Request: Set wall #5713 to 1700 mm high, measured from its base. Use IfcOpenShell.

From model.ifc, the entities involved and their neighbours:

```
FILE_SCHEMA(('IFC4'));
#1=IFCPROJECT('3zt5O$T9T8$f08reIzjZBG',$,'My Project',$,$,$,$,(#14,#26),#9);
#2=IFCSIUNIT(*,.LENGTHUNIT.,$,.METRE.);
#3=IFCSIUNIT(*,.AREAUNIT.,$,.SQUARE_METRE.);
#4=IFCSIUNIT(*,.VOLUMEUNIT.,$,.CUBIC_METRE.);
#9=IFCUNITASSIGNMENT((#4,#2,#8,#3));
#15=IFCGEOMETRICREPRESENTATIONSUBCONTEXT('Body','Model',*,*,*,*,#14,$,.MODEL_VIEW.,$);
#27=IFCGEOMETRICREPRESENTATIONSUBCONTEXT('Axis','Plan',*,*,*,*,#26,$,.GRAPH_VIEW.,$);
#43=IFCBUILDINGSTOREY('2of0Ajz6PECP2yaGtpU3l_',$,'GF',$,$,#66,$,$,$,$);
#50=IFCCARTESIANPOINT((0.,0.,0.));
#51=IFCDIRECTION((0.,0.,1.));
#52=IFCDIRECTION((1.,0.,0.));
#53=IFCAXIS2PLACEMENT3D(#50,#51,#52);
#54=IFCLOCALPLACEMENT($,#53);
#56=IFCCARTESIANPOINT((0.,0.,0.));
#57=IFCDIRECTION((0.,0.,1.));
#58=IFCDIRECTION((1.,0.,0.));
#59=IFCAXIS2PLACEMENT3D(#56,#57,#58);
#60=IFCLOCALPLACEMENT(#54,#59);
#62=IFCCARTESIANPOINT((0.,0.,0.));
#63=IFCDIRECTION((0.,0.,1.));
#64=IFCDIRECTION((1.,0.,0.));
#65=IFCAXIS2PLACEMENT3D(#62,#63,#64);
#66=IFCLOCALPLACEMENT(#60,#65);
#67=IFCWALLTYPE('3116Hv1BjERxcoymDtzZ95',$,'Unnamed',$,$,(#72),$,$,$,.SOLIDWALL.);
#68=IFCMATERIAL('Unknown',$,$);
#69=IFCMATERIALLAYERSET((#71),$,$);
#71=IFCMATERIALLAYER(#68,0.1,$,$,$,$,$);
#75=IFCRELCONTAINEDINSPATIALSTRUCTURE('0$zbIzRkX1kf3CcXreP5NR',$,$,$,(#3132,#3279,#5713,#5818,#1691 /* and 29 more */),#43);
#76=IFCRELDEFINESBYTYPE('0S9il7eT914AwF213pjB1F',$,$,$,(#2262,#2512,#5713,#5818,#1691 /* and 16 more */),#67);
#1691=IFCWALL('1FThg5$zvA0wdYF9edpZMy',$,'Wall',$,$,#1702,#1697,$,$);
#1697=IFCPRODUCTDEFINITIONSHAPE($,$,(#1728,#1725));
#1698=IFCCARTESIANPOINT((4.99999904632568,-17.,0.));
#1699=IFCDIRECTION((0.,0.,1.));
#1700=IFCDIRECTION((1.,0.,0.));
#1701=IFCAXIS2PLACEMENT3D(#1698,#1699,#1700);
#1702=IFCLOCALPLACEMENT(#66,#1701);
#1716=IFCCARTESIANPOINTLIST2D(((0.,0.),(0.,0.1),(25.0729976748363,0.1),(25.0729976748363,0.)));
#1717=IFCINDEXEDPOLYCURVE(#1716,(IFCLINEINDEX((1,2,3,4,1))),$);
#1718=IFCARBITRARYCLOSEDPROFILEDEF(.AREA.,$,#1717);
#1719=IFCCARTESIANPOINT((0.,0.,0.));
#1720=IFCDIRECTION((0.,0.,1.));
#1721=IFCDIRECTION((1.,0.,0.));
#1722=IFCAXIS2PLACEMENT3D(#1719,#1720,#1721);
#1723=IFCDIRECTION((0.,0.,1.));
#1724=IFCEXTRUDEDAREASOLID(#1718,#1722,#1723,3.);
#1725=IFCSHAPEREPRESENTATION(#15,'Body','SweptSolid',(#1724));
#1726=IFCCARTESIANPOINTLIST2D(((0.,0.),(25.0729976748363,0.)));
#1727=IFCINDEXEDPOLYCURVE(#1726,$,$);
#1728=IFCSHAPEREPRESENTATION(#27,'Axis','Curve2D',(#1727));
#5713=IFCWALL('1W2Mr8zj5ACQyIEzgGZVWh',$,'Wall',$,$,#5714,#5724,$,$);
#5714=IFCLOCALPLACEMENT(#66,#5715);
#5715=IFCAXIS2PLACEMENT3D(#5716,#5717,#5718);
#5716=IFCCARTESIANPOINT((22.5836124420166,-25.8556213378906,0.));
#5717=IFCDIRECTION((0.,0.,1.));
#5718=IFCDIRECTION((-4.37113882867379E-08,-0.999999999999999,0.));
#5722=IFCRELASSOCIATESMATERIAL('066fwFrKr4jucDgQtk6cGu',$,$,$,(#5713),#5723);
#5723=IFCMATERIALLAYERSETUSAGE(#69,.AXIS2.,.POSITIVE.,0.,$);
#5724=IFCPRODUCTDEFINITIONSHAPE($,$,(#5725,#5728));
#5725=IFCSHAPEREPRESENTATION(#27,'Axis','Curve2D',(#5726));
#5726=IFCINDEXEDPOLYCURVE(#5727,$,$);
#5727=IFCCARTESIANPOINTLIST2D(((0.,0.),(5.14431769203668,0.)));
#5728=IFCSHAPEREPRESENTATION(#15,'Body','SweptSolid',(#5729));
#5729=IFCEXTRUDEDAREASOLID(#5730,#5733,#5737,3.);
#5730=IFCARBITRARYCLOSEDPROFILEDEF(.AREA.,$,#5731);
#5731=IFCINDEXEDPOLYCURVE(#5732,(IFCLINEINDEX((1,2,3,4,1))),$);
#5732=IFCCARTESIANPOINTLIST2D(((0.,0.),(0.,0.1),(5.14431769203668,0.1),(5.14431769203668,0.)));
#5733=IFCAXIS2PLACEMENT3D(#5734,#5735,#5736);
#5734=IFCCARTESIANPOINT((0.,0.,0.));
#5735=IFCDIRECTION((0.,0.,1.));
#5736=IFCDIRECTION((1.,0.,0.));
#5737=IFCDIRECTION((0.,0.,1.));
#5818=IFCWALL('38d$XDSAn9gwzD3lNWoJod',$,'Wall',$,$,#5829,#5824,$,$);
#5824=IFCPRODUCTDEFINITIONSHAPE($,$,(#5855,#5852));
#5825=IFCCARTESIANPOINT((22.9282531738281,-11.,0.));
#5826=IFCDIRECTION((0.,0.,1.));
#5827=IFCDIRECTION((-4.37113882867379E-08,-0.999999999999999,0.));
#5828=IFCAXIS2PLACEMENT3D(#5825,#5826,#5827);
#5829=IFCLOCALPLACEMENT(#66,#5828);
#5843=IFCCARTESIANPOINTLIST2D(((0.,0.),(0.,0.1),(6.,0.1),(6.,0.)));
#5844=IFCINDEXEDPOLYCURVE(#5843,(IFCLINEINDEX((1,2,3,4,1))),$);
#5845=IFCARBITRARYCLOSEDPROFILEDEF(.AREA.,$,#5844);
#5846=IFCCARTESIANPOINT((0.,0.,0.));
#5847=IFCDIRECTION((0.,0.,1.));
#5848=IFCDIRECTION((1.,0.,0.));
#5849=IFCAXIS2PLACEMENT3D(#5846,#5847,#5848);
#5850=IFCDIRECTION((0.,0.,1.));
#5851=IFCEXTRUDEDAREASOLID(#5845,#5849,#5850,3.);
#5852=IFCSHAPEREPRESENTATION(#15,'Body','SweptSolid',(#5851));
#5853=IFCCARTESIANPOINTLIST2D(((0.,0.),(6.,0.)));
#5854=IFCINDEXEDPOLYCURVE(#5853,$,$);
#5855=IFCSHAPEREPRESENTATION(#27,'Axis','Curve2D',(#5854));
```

```python
import ifcopenshell
import ifcopenshell.geom
import ifcopenshell.util.representation
import ifcopenshell.util.shape

model = ifcopenshell.open("model.ifc")
settings = ifcopenshell.geom.settings()


def volume(element):
    """Net volume in cubic metres, openings subtracted."""
    shape = ifcopenshell.geom.create_shape(settings, element)
    return ifcopenshell.util.shape.get_volume(shape.geometry)


wall = model.by_id(5713)
before = volume(wall)

body = ifcopenshell.util.representation.get_representation(wall, "Model", "Body")
solid = body.Items[0]
old_height = solid.Depth
solid.Depth = 1.7
after = volume(wall)

print(f"height {old_height:g} -> {solid.Depth:g}, volume {before:.3f} -> {after:.3f} m3")

model.write("model_edited.ifc")
```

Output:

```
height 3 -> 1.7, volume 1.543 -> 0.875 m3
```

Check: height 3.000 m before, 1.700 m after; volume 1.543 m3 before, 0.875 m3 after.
